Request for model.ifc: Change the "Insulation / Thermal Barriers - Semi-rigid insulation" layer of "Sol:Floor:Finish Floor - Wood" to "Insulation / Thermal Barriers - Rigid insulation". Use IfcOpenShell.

First a look at what the model holds.

```python
import ifcopenshell
import ifcopenshell.util.element

model = ifcopenshell.open("model.ifc")
print(model.schema)
for layer_set in model.by_type("IfcMaterialLayerSet"):
    if layer_set.LayerSetName == "Sol:Floor:Finish Floor - Wood":
        for layer in layer_set.MaterialLayers:
            print(layer.id(), layer.Material and layer.Material.Name, layer.LayerThickness, sep=" | ")
        print(len(ifcopenshell.util.element.get_elements_by_material(model, layer_set)), "elements and types use it")
print(sorted(m.Name for m in model.by_type("IfcMaterial") if m.Name)[:60])
```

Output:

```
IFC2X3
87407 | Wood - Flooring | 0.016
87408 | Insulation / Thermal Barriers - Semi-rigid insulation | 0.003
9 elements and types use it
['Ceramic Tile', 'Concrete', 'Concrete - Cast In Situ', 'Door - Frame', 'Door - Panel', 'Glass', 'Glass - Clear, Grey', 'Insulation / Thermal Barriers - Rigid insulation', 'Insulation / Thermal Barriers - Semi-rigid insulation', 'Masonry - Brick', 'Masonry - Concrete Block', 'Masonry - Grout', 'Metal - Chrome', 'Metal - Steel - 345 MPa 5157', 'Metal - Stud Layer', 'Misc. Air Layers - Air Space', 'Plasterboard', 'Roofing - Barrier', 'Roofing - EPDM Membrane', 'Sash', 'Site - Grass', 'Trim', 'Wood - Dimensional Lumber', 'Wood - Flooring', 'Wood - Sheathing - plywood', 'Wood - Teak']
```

```python
import ifcopenshell
import ifcopenshell.api.material

model = ifcopenshell.open("model.ifc")

layer_set = next(s for s in model.by_type("IfcMaterialLayerSet") if s.LayerSetName == "Sol:Floor:Finish Floor - Wood")
layer = next(l for l in layer_set.MaterialLayers if l.Material and l.Material.Name == "Insulation / Thermal Barriers - Semi-rigid insulation")
material = next(m for m in model.by_type("IfcMaterial") if m.Name == "Insulation / Thermal Barriers - Rigid insulation")

# Point this one layer at the other material; renaming the old one would change it everywhere.
ifcopenshell.api.material.edit_layer(model, layer=layer, attributes={}, material=material)

print([l.Material.Name if l.Material else None for l in layer_set.MaterialLayers])

model.write("model_rev.ifc")
```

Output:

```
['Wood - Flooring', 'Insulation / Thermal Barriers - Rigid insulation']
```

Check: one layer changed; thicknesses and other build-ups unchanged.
